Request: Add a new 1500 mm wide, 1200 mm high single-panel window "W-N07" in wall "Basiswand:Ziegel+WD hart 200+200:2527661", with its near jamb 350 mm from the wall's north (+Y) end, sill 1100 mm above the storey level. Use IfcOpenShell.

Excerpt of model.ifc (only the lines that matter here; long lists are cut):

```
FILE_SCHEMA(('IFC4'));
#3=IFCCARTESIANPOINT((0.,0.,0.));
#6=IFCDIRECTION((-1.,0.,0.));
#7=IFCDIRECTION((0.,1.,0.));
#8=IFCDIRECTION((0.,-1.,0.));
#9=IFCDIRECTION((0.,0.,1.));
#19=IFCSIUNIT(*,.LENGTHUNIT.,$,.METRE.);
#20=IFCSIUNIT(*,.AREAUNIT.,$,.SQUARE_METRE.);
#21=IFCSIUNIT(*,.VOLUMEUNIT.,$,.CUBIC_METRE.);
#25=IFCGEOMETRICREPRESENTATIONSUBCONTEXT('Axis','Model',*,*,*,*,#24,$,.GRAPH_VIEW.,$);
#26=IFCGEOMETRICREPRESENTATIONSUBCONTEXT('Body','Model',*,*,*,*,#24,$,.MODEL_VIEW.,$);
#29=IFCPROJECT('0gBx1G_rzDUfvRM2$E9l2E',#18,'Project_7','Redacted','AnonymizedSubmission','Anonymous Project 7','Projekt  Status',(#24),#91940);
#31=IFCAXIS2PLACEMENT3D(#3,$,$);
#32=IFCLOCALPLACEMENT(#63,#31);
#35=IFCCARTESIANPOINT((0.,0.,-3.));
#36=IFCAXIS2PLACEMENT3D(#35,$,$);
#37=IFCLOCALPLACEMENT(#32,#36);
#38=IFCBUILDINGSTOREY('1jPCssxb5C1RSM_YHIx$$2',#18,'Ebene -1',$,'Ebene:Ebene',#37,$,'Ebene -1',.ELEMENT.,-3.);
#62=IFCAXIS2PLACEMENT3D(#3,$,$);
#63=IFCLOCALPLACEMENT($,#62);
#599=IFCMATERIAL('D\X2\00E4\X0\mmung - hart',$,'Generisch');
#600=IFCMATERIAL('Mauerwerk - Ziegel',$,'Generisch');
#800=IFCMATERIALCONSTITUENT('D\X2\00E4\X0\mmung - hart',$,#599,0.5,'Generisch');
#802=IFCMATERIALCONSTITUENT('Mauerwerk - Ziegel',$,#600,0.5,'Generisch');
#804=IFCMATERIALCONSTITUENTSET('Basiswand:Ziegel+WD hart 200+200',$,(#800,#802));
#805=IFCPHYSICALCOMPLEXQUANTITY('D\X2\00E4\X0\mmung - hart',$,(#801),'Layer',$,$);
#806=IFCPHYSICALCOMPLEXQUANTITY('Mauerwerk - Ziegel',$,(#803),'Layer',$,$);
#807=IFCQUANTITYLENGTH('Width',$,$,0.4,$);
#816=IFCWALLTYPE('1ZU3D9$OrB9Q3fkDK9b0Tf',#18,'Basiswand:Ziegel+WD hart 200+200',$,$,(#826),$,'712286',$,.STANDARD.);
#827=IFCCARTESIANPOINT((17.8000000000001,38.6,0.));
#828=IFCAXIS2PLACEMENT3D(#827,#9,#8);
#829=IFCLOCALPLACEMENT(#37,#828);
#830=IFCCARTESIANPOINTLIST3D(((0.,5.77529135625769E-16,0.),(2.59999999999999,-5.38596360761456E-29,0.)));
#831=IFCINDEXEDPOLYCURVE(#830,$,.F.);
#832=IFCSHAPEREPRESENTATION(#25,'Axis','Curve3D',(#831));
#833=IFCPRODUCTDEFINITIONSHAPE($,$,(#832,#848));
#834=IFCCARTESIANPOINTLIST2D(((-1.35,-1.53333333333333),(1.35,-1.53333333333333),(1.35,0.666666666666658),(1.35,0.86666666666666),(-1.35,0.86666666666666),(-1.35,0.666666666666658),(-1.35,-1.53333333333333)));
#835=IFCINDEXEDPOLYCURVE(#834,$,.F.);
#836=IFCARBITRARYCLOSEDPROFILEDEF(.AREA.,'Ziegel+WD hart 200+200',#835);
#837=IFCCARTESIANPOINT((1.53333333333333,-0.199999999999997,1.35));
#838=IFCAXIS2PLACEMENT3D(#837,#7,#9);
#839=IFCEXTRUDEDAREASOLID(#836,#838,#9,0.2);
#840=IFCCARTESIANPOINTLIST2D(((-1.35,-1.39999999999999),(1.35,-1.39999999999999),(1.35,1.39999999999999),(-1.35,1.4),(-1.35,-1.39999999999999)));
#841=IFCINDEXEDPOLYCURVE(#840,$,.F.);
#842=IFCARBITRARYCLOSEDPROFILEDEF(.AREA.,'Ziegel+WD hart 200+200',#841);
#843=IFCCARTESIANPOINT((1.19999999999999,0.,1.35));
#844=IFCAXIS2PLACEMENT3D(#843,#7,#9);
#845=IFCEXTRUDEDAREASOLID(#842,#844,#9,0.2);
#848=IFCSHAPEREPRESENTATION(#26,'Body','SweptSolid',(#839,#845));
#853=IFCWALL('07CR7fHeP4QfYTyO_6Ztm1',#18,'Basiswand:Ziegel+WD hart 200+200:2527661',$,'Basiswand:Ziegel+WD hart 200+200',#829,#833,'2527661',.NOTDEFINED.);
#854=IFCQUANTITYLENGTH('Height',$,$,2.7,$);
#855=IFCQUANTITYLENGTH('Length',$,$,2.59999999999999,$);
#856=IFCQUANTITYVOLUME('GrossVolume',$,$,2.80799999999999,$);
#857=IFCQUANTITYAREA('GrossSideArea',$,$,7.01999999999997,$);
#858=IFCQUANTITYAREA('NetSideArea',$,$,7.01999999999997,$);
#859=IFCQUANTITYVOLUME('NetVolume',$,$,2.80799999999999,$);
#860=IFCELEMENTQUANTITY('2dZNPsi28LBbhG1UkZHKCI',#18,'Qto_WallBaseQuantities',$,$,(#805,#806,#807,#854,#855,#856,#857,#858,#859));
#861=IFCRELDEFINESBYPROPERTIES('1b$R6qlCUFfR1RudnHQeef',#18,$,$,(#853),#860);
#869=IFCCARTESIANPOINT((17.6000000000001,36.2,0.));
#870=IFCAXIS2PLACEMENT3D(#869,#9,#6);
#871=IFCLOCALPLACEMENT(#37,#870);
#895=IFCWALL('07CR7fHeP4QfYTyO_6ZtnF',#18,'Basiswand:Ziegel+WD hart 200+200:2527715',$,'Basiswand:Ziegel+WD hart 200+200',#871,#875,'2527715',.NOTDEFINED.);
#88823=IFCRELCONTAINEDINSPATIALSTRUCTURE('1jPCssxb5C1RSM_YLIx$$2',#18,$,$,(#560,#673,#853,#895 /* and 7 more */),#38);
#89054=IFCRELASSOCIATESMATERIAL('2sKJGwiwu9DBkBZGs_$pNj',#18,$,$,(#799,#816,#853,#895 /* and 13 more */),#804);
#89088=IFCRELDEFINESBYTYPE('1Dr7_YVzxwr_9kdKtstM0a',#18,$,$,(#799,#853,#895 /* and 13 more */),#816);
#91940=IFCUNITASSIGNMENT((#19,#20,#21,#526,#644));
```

```python
import numpy as np
import ifcopenshell
import ifcopenshell.api.feature
import ifcopenshell.api.geometry
import ifcopenshell.api.pset
import ifcopenshell.api.root
import ifcopenshell.api.spatial
import ifcopenshell.geom
import ifcopenshell.util.element
import ifcopenshell.util.placement
import ifcopenshell.util.representation
import ifcopenshell.util.shape
import ifcopenshell.util.unit

model = ifcopenshell.open("model.ifc")
unit_scale = ifcopenshell.util.unit.calculate_unit_scale(model)
area_scale = ifcopenshell.util.unit.calculate_unit_scale(model, "AREAUNIT")
volume_scale = ifcopenshell.util.unit.calculate_unit_scale(model, "VOLUMEUNIT")
settings = ifcopenshell.geom.settings()


def volume(element):
    """Net volume in cubic metres, openings subtracted."""
    shape = ifcopenshell.geom.create_shape(settings, element)
    return ifcopenshell.util.shape.get_volume(shape.geometry)


wall = model.by_id(853)
storey = ifcopenshell.util.element.get_container(wall, ifc_class="IfcBuildingStorey")
context = ifcopenshell.util.representation.get_context(model, "Model", "Body", "MODEL_VIEW")
before = volume(wall)

width, height, from_end, sill = 1.5, 1.2, 0.35, 1.1  # metres

# The wall runs along its own X axis, and the end named is its -X end.
wall_shape = ifcopenshell.geom.create_shape(settings, wall)
x, y, z = ifcopenshell.util.shape.get_vertices(wall_shape.geometry).T
start = x.min() + from_end
face, thickness = float(y.min()), float(y.max() - y.min())
wall_matrix = ifcopenshell.util.placement.get_local_placement(wall.ObjectPlacement)
level = ifcopenshell.util.placement.get_local_placement(storey.ObjectPlacement)[2, 3]


def in_wall(x, y):
    """Placement at x, y metres in the wall's axes, at sill height."""
    matrix = wall_matrix.copy()
    matrix[:, 3] = wall_matrix @ np.array([x / unit_scale, y / unit_scale, 0.0, 1.0])
    matrix[2, 3] = level + sill / unit_scale
    return matrix


# Opening: a box that overshoots both wall faces by 50 mm.
opening = ifcopenshell.api.root.create_entity(model, ifc_class="IfcOpeningElement", predefined_type="OPENING")
box = ifcopenshell.api.geometry.add_wall_representation(
    model, context=context, length=width, height=height, thickness=thickness + 0.1
)
ifcopenshell.api.geometry.assign_representation(model, product=opening, representation=box)
ifcopenshell.api.geometry.edit_object_placement(model, product=opening, matrix=in_wall(start, face - 0.05), is_si=False)
ifcopenshell.api.feature.add_feature(model, feature=opening, element=wall)

window = ifcopenshell.api.root.create_entity(model, ifc_class="IfcWindow", name="W-N07", predefined_type="WINDOW")
window.OverallWidth, window.OverallHeight = width / unit_scale, height / unit_scale
window.PartitioningType = "SINGLE_PANEL"
body = ifcopenshell.api.geometry.add_window_representation(
    model,
    context=context,
    overall_width=window.OverallWidth,
    overall_height=window.OverallHeight,
    partition_type="SINGLE_PANEL",
)
ifcopenshell.api.geometry.assign_representation(model, product=window, representation=body)
ifcopenshell.api.spatial.assign_container(model, products=[window], relating_structure=storey)
ifcopenshell.api.feature.add_filling(model, opening=opening, element=window)

# Centre the window in the wall's thickness.
ifcopenshell.api.geometry.edit_object_placement(model, product=window, matrix=in_wall(start, face), is_si=False)
window_shape = ifcopenshell.geom.create_shape(settings, window)
depth = ifcopenshell.util.shape.get_vertices(window_shape.geometry)[:, 1]
offset = face + thickness / 2 - (depth.min() + depth.max()) / 2
ifcopenshell.api.geometry.edit_object_placement(model, product=window, matrix=in_wall(start, offset), is_si=False)

after = volume(wall)

# Update the wall's stored quantities.
qto = model.by_id(ifcopenshell.util.element.get_pset(wall, "Qto_WallBaseQuantities", should_inherit=False)["id"])
ifcopenshell.api.pset.edit_qto(model, qto=qto, properties={
    "NetSideArea": after / thickness / area_scale,
    "NetVolume": after / volume_scale,
})

print(f"wall volume {before:.3f} -> {after:.3f} m3")

model.write("model_edited.ifc")
```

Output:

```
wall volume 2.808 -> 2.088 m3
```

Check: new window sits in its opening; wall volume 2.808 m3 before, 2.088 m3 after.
